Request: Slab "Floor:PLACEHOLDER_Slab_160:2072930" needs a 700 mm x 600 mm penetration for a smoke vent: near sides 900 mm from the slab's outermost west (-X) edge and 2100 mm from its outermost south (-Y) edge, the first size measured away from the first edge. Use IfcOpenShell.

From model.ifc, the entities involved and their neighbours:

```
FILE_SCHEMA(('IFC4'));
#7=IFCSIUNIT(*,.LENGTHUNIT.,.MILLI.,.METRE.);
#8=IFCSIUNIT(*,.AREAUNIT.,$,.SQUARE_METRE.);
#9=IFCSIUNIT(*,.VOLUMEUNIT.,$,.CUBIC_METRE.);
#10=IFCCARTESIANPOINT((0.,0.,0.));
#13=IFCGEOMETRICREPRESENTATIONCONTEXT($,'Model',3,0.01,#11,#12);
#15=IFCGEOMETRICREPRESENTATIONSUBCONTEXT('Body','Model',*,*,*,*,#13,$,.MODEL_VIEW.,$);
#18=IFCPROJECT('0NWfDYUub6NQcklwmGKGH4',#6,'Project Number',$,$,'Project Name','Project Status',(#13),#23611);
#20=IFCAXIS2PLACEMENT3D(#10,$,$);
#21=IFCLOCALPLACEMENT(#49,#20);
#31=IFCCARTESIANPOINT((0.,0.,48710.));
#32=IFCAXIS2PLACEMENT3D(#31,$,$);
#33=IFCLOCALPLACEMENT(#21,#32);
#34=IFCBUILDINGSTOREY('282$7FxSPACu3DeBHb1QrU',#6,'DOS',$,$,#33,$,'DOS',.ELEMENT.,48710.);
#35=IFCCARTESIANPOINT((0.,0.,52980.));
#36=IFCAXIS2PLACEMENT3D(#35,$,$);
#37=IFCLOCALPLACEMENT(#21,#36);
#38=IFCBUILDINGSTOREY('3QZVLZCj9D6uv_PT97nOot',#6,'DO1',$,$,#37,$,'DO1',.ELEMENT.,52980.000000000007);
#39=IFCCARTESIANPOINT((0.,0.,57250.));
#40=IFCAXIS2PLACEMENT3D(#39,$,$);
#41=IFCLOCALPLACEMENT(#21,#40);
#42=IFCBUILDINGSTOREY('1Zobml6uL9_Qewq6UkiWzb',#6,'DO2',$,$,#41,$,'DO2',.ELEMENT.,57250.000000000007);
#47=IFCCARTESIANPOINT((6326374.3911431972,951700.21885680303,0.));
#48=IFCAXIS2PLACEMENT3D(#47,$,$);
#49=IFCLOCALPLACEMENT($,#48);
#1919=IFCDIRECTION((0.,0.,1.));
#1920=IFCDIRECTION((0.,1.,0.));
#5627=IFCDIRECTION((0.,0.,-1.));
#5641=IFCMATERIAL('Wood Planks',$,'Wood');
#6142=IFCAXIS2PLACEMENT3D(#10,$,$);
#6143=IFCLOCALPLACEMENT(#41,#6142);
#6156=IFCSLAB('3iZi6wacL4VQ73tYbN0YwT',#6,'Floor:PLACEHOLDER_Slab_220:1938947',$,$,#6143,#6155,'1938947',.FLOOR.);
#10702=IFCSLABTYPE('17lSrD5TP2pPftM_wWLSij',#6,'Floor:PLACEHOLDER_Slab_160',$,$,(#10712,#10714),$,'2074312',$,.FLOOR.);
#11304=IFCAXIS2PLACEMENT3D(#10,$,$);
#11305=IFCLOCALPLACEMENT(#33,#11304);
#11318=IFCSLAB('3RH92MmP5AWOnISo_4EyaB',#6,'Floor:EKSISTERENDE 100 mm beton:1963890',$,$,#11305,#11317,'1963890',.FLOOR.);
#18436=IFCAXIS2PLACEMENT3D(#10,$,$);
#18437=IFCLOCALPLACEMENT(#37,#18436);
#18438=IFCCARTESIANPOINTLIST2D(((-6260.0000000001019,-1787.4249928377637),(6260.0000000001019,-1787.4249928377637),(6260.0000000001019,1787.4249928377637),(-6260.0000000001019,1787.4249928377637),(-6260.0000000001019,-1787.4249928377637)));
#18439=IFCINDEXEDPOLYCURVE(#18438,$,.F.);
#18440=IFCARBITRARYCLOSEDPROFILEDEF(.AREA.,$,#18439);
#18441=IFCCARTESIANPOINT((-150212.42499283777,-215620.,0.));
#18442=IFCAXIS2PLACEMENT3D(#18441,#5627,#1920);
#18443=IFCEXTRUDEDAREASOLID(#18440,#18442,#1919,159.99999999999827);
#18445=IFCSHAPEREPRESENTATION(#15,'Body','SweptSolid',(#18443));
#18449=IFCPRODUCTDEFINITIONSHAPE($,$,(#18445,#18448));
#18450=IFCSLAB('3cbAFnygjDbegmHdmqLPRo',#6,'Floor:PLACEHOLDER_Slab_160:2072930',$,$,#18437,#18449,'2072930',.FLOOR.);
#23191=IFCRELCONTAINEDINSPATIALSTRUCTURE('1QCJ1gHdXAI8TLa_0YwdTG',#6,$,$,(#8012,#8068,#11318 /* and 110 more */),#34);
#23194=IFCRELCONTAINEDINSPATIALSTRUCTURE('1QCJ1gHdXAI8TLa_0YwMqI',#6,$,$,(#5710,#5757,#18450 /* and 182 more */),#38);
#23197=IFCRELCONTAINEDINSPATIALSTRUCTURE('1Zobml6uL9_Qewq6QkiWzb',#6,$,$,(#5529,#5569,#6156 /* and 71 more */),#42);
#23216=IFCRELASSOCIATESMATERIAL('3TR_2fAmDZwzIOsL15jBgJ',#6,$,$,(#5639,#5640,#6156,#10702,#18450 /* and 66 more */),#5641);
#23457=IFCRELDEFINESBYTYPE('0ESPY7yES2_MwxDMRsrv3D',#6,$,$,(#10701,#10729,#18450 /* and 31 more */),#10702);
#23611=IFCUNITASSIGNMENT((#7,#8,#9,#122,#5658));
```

```python
import numpy as np
import ifcopenshell
import ifcopenshell.api.feature
import ifcopenshell.api.geometry
import ifcopenshell.api.root
import ifcopenshell.geom
import ifcopenshell.util.placement
import ifcopenshell.util.representation
import ifcopenshell.util.shape
import ifcopenshell.util.unit

model = ifcopenshell.open("model.ifc")
unit_scale = ifcopenshell.util.unit.calculate_unit_scale(model)
settings = ifcopenshell.geom.settings()


def volume(element):
    """Net volume in cubic metres, openings subtracted."""
    shape = ifcopenshell.geom.create_shape(settings, element)
    return ifcopenshell.util.shape.get_volume(shape.geometry)


slab = model.by_guid("3cbAFnygjDbegmHdmqLPRo")
before = volume(slab)

# Extent in the slab's own axes, in metres. The edges named are its -X and -Y sides.
slab_shape = ifcopenshell.geom.create_shape(settings, slab)
vertices = ifcopenshell.util.shape.get_vertices(slab_shape.geometry)
x_min, y_min, bottom = vertices.min(axis=0)
top = vertices[:, 2].max()

opening = ifcopenshell.api.root.create_entity(model, ifc_class="IfcOpeningElement", name="Smoke vent opening", predefined_type="OPENING")
context = ifcopenshell.util.representation.get_context(model, "Model", "Body", "MODEL_VIEW")
width, depth = 0.7, 0.6
outline = [(0.0, 0.0), (width, 0.0), (width, depth), (0.0, depth), (0.0, 0.0)]
# Overshoot both faces by 50 mm so the cut is clean.
shape = ifcopenshell.api.geometry.add_slab_representation(
    model, context=context, depth=top - bottom + 0.1, polyline=outline
)
ifcopenshell.api.geometry.assign_representation(model, product=opening, representation=shape)

matrix = ifcopenshell.util.placement.get_local_placement(slab.ObjectPlacement)
matrix[:, 3] = matrix @ np.append(np.array([x_min + 0.9, y_min + 2.1, bottom - 0.05]) / unit_scale, 1.0)
ifcopenshell.api.geometry.edit_object_placement(model, product=opening, matrix=matrix, is_si=False)
ifcopenshell.api.feature.add_feature(model, feature=opening, element=slab)

after = volume(slab)

print(f"slab volume {before:.3f} -> {after:.3f} m3")

model.write("model_edited.ifc")
```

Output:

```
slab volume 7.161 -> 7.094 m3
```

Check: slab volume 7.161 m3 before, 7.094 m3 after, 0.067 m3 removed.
